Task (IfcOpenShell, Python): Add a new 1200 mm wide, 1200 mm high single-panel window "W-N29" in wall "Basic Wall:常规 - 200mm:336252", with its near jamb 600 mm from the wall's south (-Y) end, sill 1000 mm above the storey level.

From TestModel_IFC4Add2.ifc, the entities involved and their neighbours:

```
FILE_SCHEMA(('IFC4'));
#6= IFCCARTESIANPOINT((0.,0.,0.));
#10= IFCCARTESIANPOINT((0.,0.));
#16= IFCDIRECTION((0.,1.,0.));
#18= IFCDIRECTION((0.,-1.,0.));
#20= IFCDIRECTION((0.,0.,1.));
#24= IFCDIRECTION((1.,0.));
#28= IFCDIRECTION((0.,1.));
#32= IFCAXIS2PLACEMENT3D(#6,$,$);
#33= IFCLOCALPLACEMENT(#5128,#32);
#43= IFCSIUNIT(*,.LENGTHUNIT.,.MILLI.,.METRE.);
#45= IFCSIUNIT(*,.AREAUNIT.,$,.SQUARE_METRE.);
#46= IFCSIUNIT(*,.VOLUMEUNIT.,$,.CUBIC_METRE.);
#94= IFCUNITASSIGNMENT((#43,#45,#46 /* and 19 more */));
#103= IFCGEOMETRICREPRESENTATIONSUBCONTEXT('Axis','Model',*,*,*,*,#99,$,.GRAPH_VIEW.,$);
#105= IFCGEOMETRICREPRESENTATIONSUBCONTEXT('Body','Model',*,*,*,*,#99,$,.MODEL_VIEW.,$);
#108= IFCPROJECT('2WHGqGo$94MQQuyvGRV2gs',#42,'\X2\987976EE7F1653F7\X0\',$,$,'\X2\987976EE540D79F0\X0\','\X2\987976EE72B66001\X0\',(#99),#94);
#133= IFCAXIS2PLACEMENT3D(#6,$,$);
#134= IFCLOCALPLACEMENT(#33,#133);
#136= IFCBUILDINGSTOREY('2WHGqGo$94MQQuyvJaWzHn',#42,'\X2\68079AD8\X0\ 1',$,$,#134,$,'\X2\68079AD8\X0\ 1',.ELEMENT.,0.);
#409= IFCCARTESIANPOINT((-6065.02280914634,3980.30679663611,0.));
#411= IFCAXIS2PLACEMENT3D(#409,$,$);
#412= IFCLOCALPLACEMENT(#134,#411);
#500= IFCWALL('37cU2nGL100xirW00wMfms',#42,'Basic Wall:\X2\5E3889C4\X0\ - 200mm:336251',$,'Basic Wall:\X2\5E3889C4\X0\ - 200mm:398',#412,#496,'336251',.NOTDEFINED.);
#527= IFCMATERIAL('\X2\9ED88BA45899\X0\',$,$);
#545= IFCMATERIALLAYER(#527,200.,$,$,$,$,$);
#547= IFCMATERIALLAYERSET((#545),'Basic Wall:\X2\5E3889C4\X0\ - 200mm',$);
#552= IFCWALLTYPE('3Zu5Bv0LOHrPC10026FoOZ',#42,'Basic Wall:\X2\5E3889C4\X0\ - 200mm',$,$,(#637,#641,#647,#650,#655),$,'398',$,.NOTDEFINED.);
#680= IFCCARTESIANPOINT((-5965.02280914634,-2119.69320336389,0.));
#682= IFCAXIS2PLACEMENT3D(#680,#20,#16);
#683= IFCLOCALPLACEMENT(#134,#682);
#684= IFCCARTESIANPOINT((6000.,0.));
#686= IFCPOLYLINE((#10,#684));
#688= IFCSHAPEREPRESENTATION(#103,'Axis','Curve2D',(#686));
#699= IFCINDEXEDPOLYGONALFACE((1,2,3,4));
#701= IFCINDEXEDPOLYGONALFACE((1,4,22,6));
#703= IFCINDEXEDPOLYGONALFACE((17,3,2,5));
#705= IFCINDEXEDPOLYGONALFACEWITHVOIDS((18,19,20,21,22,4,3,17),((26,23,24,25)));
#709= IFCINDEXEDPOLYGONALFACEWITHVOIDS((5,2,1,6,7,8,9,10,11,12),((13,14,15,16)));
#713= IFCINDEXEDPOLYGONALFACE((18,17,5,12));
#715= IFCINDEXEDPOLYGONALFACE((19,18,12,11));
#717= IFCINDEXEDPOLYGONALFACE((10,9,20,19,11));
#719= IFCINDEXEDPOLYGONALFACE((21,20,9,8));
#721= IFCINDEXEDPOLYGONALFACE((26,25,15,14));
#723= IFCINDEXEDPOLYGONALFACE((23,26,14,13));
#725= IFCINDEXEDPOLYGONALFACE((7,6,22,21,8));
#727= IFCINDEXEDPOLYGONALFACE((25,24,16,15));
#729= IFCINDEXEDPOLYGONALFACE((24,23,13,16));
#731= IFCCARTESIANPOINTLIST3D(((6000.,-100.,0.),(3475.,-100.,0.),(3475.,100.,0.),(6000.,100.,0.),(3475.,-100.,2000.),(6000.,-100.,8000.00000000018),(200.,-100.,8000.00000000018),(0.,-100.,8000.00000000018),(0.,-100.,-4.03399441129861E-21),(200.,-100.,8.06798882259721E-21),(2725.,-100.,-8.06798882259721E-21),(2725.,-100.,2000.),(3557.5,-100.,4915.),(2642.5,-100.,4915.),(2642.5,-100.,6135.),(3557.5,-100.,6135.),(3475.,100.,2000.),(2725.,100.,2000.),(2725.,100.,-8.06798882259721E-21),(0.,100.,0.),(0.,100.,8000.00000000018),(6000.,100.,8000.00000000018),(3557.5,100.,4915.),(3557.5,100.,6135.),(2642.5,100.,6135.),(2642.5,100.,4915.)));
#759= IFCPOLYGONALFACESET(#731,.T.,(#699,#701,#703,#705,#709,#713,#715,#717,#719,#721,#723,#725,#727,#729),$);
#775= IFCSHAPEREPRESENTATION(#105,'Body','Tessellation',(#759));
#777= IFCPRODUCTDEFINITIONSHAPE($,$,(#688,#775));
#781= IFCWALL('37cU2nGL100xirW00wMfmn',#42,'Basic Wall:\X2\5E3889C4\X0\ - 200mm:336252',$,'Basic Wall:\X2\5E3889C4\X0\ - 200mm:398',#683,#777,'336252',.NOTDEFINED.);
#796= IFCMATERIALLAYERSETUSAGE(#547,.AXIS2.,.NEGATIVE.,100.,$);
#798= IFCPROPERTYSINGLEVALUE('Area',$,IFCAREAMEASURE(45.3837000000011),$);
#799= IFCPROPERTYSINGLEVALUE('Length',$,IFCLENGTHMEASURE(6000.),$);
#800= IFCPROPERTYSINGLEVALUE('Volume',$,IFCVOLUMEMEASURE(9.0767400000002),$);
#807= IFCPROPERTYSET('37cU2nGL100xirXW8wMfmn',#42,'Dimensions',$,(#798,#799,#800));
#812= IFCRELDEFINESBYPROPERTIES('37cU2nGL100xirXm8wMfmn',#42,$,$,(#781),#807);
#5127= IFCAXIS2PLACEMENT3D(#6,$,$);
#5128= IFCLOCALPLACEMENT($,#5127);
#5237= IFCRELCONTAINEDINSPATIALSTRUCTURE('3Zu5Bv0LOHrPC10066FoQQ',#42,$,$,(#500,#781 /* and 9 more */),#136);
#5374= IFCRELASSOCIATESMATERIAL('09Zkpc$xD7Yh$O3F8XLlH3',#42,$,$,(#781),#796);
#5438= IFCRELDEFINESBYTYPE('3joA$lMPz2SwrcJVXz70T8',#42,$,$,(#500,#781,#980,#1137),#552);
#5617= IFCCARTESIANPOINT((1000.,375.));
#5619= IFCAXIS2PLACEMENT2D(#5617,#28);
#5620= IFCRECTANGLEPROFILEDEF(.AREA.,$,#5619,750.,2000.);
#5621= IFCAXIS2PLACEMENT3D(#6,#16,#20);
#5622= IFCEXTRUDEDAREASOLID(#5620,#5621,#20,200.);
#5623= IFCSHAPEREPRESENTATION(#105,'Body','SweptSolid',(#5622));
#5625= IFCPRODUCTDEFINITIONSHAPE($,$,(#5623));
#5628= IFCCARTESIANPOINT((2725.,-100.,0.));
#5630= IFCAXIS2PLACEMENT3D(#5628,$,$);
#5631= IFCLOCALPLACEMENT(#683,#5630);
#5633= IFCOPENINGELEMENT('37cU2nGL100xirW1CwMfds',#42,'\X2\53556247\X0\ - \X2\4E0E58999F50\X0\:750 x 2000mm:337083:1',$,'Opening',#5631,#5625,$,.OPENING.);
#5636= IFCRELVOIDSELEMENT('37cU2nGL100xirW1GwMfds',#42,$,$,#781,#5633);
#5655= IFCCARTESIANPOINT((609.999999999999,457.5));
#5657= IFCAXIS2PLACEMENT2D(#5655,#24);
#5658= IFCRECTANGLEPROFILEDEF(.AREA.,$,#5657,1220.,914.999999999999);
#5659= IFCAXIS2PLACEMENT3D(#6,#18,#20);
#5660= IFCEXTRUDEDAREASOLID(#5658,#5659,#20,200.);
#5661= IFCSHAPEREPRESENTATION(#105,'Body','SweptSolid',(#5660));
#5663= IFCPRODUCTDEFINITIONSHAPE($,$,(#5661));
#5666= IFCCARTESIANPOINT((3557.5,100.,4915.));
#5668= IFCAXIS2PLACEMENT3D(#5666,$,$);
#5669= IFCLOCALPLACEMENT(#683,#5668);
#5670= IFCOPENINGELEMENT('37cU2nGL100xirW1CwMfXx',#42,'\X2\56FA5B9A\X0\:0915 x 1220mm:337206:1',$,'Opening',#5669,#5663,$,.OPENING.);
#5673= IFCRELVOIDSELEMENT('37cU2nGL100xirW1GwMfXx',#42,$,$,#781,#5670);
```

```python
import numpy as np
import ifcopenshell
import ifcopenshell.api.feature
import ifcopenshell.api.geometry
import ifcopenshell.api.pset
import ifcopenshell.api.root
import ifcopenshell.api.spatial
import ifcopenshell.geom
import ifcopenshell.util.element
import ifcopenshell.util.placement
import ifcopenshell.util.representation
import ifcopenshell.util.shape
import ifcopenshell.util.unit

model = ifcopenshell.open("TestModel_IFC4Add2.ifc")
unit_scale = ifcopenshell.util.unit.calculate_unit_scale(model)
area_scale = ifcopenshell.util.unit.calculate_unit_scale(model, "AREAUNIT")
volume_scale = ifcopenshell.util.unit.calculate_unit_scale(model, "VOLUMEUNIT")
settings = ifcopenshell.geom.settings()


def volume(element):
    """Net volume in cubic metres, openings subtracted."""
    shape = ifcopenshell.geom.create_shape(settings, element)
    return ifcopenshell.util.shape.get_volume(shape.geometry)


wall = model.by_guid("37cU2nGL100xirW00wMfmn")
storey = ifcopenshell.util.element.get_container(wall, ifc_class="IfcBuildingStorey")
context = ifcopenshell.util.representation.get_context(model, "Model", "Body", "MODEL_VIEW")
before = volume(wall)

width, height, from_end, sill = 1.2, 1.2, 0.6, 1  # metres

# The wall runs along its own X axis, and the end named is its -X end.
wall_shape = ifcopenshell.geom.create_shape(settings, wall)
x, y, z = ifcopenshell.util.shape.get_vertices(wall_shape.geometry).T
start = x.min() + from_end
face, thickness = float(y.min()), float(y.max() - y.min())
wall_matrix = ifcopenshell.util.placement.get_local_placement(wall.ObjectPlacement)
level = ifcopenshell.util.placement.get_local_placement(storey.ObjectPlacement)[2, 3]


def in_wall(x, y):
    """Placement at x, y metres in the wall's axes, at sill height."""
    matrix = wall_matrix.copy()
    matrix[:, 3] = wall_matrix @ np.array([x / unit_scale, y / unit_scale, 0.0, 1.0])
    matrix[2, 3] = level + sill / unit_scale
    return matrix


# Opening: a box that overshoots both wall faces by 50 mm.
opening = ifcopenshell.api.root.create_entity(model, ifc_class="IfcOpeningElement", predefined_type="OPENING")
box = ifcopenshell.api.geometry.add_wall_representation(
    model, context=context, length=width, height=height, thickness=thickness + 0.1
)
ifcopenshell.api.geometry.assign_representation(model, product=opening, representation=box)
ifcopenshell.api.geometry.edit_object_placement(model, product=opening, matrix=in_wall(start, face - 0.05), is_si=False)
ifcopenshell.api.feature.add_feature(model, feature=opening, element=wall)

window = ifcopenshell.api.root.create_entity(model, ifc_class="IfcWindow", name="W-N29", predefined_type="WINDOW")
window.OverallWidth, window.OverallHeight = width / unit_scale, height / unit_scale
window.PartitioningType = "SINGLE_PANEL"
body = ifcopenshell.api.geometry.add_window_representation(
    model,
    context=context,
    overall_width=window.OverallWidth,
    overall_height=window.OverallHeight,
    partition_type="SINGLE_PANEL",
)
ifcopenshell.api.geometry.assign_representation(model, product=window, representation=body)
ifcopenshell.api.spatial.assign_container(model, products=[window], relating_structure=storey)
ifcopenshell.api.feature.add_filling(model, opening=opening, element=window)

# Centre the window in the wall's thickness.
ifcopenshell.api.geometry.edit_object_placement(model, product=window, matrix=in_wall(start, face), is_si=False)
window_shape = ifcopenshell.geom.create_shape(settings, window)
depth = ifcopenshell.util.shape.get_vertices(window_shape.geometry)[:, 1]
offset = face + thickness / 2 - (depth.min() + depth.max()) / 2
ifcopenshell.api.geometry.edit_object_placement(model, product=window, matrix=in_wall(start, offset), is_si=False)

after = volume(wall)

# Update the wall's stored quantities.
pset = model.by_id(ifcopenshell.util.element.get_pset(wall, "Dimensions", should_inherit=False)["id"])
ifcopenshell.api.pset.edit_pset(model, pset=pset, properties={
    "Area": model.create_entity("IfcAreaMeasure", after / thickness / area_scale),
    "Volume": model.create_entity("IfcVolumeMeasure", after / volume_scale),
})

print(f"wall volume {before:.3f} -> {after:.3f} m3")

model.write("TestModel_IFC4Add2_rev.ifc")
```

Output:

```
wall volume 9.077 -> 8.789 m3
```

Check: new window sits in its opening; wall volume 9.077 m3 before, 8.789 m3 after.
